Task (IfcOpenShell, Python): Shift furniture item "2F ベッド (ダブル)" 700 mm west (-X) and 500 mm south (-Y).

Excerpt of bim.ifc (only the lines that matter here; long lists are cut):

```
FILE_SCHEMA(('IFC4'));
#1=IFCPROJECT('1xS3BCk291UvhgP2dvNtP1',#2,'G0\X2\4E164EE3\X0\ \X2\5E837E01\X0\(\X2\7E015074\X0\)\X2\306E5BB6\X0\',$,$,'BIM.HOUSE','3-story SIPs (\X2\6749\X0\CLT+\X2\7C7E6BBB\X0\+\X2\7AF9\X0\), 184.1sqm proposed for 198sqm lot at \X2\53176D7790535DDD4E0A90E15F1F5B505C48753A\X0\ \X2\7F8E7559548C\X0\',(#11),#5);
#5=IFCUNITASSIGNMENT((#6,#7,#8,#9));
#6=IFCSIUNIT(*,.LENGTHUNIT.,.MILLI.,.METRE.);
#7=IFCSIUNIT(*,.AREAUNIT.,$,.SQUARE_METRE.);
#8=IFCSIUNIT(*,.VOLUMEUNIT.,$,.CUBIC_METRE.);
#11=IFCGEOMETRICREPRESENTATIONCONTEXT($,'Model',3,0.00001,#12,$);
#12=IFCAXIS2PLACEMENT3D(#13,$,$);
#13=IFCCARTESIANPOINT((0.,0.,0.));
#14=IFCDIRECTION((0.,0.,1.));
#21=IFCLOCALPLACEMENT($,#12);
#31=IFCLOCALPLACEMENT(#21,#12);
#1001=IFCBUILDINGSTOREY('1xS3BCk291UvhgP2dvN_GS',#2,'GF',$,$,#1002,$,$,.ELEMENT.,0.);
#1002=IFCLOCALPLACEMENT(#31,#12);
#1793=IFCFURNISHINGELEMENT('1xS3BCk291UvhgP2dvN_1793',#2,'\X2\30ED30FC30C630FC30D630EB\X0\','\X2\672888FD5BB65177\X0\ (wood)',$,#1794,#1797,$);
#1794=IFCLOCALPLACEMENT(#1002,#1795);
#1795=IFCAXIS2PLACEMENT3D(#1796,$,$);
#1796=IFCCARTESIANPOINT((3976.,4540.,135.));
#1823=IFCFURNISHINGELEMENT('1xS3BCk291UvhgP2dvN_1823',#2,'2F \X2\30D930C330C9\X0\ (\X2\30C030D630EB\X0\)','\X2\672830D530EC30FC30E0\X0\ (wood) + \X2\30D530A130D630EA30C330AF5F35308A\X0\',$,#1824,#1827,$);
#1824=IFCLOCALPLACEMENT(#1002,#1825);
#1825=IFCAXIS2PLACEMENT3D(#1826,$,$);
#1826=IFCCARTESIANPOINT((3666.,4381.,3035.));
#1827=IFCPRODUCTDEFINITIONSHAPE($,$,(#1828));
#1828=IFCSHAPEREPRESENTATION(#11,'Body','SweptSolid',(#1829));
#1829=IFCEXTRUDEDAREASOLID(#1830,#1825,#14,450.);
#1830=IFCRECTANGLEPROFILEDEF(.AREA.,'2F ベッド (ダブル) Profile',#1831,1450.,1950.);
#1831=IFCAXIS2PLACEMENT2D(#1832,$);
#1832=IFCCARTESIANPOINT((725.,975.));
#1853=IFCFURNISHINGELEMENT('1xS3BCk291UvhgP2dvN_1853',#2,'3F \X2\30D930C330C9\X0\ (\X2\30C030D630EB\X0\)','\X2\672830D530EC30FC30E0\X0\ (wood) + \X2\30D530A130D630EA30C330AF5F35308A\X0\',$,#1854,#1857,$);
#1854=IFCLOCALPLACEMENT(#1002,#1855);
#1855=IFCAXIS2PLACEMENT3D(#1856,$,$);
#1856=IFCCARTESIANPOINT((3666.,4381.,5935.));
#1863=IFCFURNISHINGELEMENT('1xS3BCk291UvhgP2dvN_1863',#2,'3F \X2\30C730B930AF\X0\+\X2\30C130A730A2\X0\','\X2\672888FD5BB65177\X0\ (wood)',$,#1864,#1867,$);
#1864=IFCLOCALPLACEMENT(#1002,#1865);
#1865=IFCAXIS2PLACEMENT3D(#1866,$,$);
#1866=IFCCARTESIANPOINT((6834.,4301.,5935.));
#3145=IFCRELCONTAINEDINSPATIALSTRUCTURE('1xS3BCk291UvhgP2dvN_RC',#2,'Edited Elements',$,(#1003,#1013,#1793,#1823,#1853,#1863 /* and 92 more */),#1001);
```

```python
import ifcopenshell
import ifcopenshell.api.geometry
import ifcopenshell.util.placement
import ifcopenshell.util.unit

model = ifcopenshell.open("bim.ifc")
unit_scale = ifcopenshell.util.unit.calculate_unit_scale(model)

item = model.by_guid("1xS3BCk291UvhgP2dvN_1823")
matrix = ifcopenshell.util.placement.get_local_placement(item.ObjectPlacement)
matrix[0, 3] -= 0.7 / unit_scale
matrix[1, 3] -= 0.5 / unit_scale
ifcopenshell.api.geometry.edit_object_placement(model, product=item, matrix=matrix, is_si=False)

print(ifcopenshell.util.placement.get_local_placement(item.ObjectPlacement).round(3) + 0.0)

model.write("bim_updated.ifc")
```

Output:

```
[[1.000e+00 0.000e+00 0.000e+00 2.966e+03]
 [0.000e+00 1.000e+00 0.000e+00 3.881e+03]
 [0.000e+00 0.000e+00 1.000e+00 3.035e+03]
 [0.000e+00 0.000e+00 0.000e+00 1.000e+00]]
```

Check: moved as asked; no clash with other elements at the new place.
